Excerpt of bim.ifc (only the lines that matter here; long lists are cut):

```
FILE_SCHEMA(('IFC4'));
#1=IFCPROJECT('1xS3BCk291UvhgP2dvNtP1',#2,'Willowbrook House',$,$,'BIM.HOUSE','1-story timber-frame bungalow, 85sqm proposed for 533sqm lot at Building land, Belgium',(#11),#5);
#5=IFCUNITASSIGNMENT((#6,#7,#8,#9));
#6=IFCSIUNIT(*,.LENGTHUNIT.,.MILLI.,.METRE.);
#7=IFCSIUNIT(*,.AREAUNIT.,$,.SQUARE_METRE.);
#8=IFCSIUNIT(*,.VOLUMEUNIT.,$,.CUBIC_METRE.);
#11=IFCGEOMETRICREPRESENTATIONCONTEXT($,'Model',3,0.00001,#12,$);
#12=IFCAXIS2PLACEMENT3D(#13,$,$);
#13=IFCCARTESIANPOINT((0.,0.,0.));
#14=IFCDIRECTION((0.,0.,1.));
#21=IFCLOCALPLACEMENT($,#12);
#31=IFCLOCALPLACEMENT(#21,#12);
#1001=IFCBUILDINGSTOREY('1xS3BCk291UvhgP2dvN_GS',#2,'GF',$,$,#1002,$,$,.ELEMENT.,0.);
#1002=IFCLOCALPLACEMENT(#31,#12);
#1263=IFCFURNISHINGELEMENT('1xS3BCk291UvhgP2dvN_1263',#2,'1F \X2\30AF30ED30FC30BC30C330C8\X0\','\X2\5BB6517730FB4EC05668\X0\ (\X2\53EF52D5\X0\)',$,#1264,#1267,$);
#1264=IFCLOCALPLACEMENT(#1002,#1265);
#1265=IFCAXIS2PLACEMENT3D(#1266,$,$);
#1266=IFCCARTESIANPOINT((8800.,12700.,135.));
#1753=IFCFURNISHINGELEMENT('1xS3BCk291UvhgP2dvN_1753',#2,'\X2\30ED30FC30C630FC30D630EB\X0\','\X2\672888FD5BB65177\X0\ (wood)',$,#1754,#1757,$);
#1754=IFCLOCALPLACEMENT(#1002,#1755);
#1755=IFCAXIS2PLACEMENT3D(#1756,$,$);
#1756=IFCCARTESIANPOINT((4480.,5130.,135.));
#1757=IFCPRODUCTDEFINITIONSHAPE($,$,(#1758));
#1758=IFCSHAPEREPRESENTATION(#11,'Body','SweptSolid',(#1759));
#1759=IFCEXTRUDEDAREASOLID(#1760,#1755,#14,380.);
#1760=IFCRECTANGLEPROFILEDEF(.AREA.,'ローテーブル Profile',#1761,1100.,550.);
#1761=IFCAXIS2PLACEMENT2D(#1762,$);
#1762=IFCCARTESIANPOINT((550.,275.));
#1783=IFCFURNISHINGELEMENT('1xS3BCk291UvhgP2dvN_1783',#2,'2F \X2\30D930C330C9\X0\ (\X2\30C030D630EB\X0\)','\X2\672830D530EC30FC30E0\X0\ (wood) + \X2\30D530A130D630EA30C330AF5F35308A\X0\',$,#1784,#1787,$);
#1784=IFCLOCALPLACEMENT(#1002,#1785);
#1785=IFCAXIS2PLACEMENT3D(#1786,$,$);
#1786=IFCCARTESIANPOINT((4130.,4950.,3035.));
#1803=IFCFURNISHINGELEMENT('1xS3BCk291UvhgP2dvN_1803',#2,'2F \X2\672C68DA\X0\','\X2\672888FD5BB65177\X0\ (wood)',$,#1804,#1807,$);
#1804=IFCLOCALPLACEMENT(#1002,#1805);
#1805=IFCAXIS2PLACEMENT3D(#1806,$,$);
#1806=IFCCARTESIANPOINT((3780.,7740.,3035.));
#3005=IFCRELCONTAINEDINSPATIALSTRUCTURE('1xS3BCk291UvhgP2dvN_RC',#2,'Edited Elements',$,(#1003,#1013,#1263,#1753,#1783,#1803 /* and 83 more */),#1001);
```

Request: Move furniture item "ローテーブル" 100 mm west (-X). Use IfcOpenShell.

```python
import ifcopenshell
import ifcopenshell.api.geometry
import ifcopenshell.util.placement

model = ifcopenshell.open("bim.ifc")

item = model.by_id(1753)
matrix = ifcopenshell.util.placement.get_local_placement(item.ObjectPlacement)
matrix[0, 3] -= 100.0
ifcopenshell.api.geometry.edit_object_placement(model, product=item, matrix=matrix, is_si=False)

print(ifcopenshell.util.placement.get_local_placement(item.ObjectPlacement).round(3) + 0.0)

model.write("bim_rev.ifc")
```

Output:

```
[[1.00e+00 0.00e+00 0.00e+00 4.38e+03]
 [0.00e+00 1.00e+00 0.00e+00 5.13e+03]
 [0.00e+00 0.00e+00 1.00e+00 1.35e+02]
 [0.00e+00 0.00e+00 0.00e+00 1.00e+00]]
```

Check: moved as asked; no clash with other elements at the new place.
